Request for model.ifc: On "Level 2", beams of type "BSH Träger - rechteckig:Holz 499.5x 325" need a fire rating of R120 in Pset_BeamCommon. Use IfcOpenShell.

First a look at what the model holds.

```python
import ifcopenshell
import ifcopenshell.util.element

model = ifcopenshell.open("model.ifc")
print(model.schema)
storey = next(s for s in model.by_type("IfcBuildingStorey") if s.Name == "Level 2")
beams = [e for e in ifcopenshell.util.element.get_decomposition(storey) if e.is_a("IfcBeam")]
seen = {}
for e in beams:
    element_type = ifcopenshell.util.element.get_type(e)
    key = (element_type.Name if element_type != e and element_type else None, ifcopenshell.util.element.get_pset(e, "Pset_BeamCommon", "FireRating"))
    seen[key] = seen.get(key, 0) + 1
for (name, value), count in sorted(seen.items(), key=str):
    print(count, "x", name, "|", value)
```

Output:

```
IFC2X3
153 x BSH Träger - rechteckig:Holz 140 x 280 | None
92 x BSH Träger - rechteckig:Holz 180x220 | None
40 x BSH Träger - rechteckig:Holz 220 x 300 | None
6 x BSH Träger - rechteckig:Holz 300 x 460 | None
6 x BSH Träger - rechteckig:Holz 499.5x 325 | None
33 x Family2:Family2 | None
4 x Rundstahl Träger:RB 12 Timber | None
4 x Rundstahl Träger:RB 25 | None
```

```python
import ifcopenshell
import ifcopenshell.api.pset
import ifcopenshell.util.element

model = ifcopenshell.open("model.ifc")

storey = next(s for s in model.by_type("IfcBuildingStorey") if s.Name == "Level 2")
beams = [e for e in ifcopenshell.util.element.get_decomposition(storey) if e.is_a("IfcBeam")]

count = 0
for e in beams:
    element_type = ifcopenshell.util.element.get_type(e)
    if element_type in (None, e) or element_type.Name != "BSH Träger - rechteckig:Holz 499.5x 325":
        continue
    # add_pset returns the element's existing set when there is one.
    pset = ifcopenshell.api.pset.add_pset(model, product=e, name="Pset_BeamCommon")
    ifcopenshell.api.pset.edit_pset(model, pset=pset, properties={"FireRating": "R120"})
    count += 1

print(count, "beams updated")

model.write("model_v2.ifc")
```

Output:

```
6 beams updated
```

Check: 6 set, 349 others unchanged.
